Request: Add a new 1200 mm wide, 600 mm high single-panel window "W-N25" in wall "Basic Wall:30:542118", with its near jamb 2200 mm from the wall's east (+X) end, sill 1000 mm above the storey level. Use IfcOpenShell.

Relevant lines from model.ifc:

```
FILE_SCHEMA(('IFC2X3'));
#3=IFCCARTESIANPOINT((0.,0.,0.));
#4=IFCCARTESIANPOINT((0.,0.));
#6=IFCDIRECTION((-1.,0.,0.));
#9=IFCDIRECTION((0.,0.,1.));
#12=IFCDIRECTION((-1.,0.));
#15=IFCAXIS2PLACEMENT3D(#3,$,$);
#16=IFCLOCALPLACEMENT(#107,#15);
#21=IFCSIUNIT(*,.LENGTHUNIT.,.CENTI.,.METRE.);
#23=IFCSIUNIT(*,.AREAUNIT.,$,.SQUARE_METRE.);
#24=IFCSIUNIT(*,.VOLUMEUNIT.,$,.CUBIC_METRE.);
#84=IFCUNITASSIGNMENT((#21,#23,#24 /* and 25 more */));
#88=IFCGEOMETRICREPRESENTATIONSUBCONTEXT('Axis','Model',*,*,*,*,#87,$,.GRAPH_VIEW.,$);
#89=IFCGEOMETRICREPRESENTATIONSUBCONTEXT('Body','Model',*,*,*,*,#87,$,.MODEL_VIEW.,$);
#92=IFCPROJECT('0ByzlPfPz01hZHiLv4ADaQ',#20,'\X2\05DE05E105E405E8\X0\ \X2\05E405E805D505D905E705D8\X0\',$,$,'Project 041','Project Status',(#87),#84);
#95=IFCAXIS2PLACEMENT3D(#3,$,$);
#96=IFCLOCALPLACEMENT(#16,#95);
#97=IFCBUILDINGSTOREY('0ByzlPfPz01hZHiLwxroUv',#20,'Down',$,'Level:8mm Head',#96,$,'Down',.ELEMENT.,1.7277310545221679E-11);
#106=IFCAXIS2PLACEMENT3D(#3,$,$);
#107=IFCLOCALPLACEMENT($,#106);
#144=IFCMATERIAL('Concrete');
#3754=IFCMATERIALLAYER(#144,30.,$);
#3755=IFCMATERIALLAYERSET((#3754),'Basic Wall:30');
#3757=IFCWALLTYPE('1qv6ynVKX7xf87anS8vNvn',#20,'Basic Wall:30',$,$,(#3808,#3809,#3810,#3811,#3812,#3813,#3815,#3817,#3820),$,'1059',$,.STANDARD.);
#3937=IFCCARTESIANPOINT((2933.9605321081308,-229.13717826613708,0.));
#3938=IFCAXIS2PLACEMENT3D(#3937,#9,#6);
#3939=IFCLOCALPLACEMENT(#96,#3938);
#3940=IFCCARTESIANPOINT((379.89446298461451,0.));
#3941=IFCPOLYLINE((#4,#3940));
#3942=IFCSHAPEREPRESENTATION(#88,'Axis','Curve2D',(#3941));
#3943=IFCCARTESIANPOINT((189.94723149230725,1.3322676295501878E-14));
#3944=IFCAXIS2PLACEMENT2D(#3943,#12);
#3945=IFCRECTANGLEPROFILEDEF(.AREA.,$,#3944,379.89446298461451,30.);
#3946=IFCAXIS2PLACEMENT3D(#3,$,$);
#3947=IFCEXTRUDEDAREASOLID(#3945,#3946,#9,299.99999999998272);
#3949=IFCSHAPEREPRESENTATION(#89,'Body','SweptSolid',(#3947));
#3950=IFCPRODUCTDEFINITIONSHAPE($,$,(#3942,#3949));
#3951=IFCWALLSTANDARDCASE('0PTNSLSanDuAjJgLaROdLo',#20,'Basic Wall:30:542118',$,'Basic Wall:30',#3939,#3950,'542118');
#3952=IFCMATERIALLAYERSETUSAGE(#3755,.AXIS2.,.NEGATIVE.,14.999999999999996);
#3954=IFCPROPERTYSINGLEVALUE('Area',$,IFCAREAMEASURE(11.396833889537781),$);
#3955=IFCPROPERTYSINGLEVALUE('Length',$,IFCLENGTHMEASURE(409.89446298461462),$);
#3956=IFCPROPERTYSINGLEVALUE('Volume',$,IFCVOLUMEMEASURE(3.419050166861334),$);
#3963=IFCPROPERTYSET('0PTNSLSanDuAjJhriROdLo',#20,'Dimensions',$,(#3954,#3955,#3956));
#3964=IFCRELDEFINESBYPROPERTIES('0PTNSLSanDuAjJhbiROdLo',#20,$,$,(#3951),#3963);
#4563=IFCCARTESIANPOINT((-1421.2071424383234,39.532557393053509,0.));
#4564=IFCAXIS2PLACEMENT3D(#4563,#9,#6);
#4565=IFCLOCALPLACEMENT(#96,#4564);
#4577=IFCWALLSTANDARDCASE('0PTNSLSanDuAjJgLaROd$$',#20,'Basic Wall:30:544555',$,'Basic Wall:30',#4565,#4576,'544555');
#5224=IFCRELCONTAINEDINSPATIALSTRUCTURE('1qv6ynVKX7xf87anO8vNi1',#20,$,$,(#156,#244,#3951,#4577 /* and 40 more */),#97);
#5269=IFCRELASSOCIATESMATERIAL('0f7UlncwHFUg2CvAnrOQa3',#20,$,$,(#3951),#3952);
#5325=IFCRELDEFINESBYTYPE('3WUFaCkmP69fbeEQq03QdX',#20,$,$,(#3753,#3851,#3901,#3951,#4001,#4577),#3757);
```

```python
import numpy as np
import ifcopenshell
import ifcopenshell.api.feature
import ifcopenshell.api.geometry
import ifcopenshell.api.pset
import ifcopenshell.api.root
import ifcopenshell.api.spatial
import ifcopenshell.api.type
import ifcopenshell.geom
import ifcopenshell.util.element
import ifcopenshell.util.placement
import ifcopenshell.util.representation
import ifcopenshell.util.shape
import ifcopenshell.util.unit

model = ifcopenshell.open("model.ifc")
unit_scale = ifcopenshell.util.unit.calculate_unit_scale(model)
area_scale = ifcopenshell.util.unit.calculate_unit_scale(model, "AREAUNIT")
volume_scale = ifcopenshell.util.unit.calculate_unit_scale(model, "VOLUMEUNIT")
settings = ifcopenshell.geom.settings()


def volume(element):
    """Net volume in cubic metres, openings subtracted."""
    shape = ifcopenshell.geom.create_shape(settings, element)
    return ifcopenshell.util.shape.get_volume(shape.geometry)


wall = model.by_guid("0PTNSLSanDuAjJgLaROdLo")
storey = ifcopenshell.util.element.get_container(wall, ifc_class="IfcBuildingStorey")
context = ifcopenshell.util.representation.get_context(model, "Model", "Body", "MODEL_VIEW")
before = volume(wall)

width, height, from_end, sill = 1.2, 0.6, 2.2, 1  # metres

# The wall runs along its own X axis, and the end named is its -X end.
wall_shape = ifcopenshell.geom.create_shape(settings, wall)
x, y, z = ifcopenshell.util.shape.get_vertices(wall_shape.geometry).T
start = x.min() + from_end
face, thickness = float(y.min()), float(y.max() - y.min())
wall_matrix = ifcopenshell.util.placement.get_local_placement(wall.ObjectPlacement)
level = ifcopenshell.util.placement.get_local_placement(storey.ObjectPlacement)[2, 3]


def in_wall(x, y):
    """Placement at x, y metres in the wall's axes, at sill height."""
    matrix = wall_matrix.copy()
    matrix[:, 3] = wall_matrix @ np.array([x / unit_scale, y / unit_scale, 0.0, 1.0])
    matrix[2, 3] = level + sill / unit_scale
    return matrix


# Opening: a box that overshoots both wall faces by 50 mm.
opening = ifcopenshell.api.root.create_entity(model, ifc_class="IfcOpeningElement")
box = ifcopenshell.api.geometry.add_wall_representation(
    model, context=context, length=width, height=height, thickness=thickness + 0.1
)
ifcopenshell.api.geometry.assign_representation(model, product=opening, representation=box)
ifcopenshell.api.geometry.edit_object_placement(model, product=opening, matrix=in_wall(start, face - 0.05), is_si=False)
ifcopenshell.api.feature.add_feature(model, feature=opening, element=wall)

window = ifcopenshell.api.root.create_entity(model, ifc_class="IfcWindow", name="W-N25")
window.OverallWidth, window.OverallHeight = width / unit_scale, height / unit_scale
body = ifcopenshell.api.geometry.add_window_representation(
    model,
    context=context,
    overall_width=window.OverallWidth,
    overall_height=window.OverallHeight,
    partition_type="SINGLE_PANEL",
)
ifcopenshell.api.geometry.assign_representation(model, product=window, representation=body)
ifcopenshell.api.spatial.assign_container(model, products=[window], relating_structure=storey)
fills = ifcopenshell.api.feature.add_filling(model, opening=opening, element=window)
fills.OwnerHistory = window.OwnerHistory  # required in IFC2X3

# IFC2X3 keeps the operation on the window style.
style = ifcopenshell.api.root.create_entity(model, ifc_class="IfcWindowStyle", name="W-N25")
style.OperationType, style.ConstructionType = "SINGLE_PANEL", "NOTDEFINED"
style.ParameterTakesPrecedence = style.Sizeable = False
ifcopenshell.api.type.assign_type(model, related_objects=[window], relating_type=style)

# Centre the window in the wall's thickness.
ifcopenshell.api.geometry.edit_object_placement(model, product=window, matrix=in_wall(start, face), is_si=False)
window_shape = ifcopenshell.geom.create_shape(settings, window)
depth = ifcopenshell.util.shape.get_vertices(window_shape.geometry)[:, 1]
offset = face + thickness / 2 - (depth.min() + depth.max()) / 2
ifcopenshell.api.geometry.edit_object_placement(model, product=window, matrix=in_wall(start, offset), is_si=False)

after = volume(wall)

# Update the wall's stored quantities.
pset = model.by_id(ifcopenshell.util.element.get_pset(wall, "Dimensions", should_inherit=False)["id"])
ifcopenshell.api.pset.edit_pset(model, pset=pset, properties={
    "Area": model.create_entity("IfcAreaMeasure", after / thickness / area_scale),
    "Volume": model.create_entity("IfcVolumeMeasure", after / volume_scale),
})

print(f"wall volume {before:.3f} -> {after:.3f} m3")

model.write("model_v2.ifc")
```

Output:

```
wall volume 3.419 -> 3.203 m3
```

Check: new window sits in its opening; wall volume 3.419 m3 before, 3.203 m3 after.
